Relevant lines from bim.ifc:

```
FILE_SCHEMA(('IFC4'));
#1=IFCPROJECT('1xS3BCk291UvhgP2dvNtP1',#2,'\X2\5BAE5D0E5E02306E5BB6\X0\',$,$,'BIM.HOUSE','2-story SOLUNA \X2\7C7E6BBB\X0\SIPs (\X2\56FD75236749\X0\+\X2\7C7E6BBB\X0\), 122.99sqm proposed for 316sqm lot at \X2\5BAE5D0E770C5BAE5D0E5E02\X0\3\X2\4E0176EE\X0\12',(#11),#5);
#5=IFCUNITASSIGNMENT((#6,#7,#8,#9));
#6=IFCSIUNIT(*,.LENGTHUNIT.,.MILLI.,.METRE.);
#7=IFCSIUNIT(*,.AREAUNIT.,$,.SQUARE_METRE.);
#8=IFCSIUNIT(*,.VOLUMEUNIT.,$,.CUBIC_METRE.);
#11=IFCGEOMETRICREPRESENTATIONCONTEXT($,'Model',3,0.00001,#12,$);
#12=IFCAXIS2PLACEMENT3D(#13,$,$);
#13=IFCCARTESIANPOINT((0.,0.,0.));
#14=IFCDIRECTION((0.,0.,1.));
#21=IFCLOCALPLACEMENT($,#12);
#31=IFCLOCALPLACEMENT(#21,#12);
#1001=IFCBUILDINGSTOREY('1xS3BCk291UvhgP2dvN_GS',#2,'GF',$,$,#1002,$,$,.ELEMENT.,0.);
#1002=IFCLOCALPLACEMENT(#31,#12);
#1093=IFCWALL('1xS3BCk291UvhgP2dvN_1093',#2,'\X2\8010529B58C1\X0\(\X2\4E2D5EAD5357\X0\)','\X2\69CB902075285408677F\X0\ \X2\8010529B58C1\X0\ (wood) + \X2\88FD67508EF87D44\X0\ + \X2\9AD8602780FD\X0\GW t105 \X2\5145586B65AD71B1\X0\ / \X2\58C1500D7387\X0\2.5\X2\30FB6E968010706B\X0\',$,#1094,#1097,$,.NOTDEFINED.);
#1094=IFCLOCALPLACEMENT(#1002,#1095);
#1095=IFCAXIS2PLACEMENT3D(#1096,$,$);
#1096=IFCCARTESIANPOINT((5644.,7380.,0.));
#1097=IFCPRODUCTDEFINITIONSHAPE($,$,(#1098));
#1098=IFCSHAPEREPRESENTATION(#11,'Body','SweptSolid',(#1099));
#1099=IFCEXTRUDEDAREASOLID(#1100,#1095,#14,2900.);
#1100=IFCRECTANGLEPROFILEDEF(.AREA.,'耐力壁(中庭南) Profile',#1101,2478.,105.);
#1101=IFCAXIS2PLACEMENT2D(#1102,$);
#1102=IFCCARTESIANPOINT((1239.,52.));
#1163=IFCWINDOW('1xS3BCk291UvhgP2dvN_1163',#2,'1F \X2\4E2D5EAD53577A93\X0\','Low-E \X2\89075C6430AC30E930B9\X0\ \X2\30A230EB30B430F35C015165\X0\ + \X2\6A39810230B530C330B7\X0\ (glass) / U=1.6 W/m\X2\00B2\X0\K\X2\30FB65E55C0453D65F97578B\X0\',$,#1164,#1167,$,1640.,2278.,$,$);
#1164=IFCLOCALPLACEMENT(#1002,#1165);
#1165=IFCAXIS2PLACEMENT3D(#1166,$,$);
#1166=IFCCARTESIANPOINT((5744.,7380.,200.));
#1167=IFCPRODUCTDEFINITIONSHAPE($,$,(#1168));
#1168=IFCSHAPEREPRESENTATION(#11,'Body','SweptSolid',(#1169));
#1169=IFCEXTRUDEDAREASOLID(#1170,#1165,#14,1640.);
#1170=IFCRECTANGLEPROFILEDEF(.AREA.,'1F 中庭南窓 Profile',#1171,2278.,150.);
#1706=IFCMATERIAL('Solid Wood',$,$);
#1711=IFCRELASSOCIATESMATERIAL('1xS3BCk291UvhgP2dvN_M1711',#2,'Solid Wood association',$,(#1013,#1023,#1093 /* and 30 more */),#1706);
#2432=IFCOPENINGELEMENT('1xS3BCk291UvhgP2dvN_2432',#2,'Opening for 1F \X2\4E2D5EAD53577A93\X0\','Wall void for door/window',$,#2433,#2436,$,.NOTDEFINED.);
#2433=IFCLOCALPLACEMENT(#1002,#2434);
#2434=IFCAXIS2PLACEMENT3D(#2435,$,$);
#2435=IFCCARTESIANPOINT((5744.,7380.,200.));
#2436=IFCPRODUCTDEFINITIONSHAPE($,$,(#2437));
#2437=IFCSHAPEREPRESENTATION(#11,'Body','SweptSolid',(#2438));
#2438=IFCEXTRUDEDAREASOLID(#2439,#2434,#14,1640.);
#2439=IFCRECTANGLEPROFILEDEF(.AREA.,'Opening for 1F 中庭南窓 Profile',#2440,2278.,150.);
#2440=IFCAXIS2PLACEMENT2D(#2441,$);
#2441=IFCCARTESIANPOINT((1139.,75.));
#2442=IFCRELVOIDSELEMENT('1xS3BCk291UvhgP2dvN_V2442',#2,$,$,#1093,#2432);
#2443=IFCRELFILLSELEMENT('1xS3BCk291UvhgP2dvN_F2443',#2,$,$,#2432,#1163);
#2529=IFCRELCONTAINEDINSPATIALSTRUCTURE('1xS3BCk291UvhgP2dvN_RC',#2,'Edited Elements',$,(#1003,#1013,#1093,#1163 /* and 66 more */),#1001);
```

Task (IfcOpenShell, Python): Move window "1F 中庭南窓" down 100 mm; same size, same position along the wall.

```python
import numpy as np
import ifcopenshell
import ifcopenshell.api.geometry
import ifcopenshell.util.placement
import ifcopenshell.util.unit

model = ifcopenshell.open("bim.ifc")
unit_scale = ifcopenshell.util.unit.calculate_unit_scale(model)

window = model.by_guid("1xS3BCk291UvhgP2dvN_1163")
opening = window.FillsVoids[0].RelatingOpeningElement
dz = -0.1 / unit_scale

shift = np.array([0.0, 0.0, dz])
# The window is not placed relative to its opening, so move both.
for product in (opening, window):
    matrix = ifcopenshell.util.placement.get_local_placement(product.ObjectPlacement)
    matrix[:3, 3] += shift
    ifcopenshell.api.geometry.edit_object_placement(model, product=product, matrix=matrix, is_si=False)

print(f"moved by {dz * unit_scale:+.3f} m")

model.write("bim_updated.ifc")
```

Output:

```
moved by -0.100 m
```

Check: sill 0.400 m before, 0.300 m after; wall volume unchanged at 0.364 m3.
